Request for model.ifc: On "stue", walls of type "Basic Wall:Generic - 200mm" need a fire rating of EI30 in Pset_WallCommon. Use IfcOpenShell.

First a look at what the model holds.

```python
import ifcopenshell
import ifcopenshell.util.element

model = ifcopenshell.open("model.ifc")
print(model.schema)
storey = next(s for s in model.by_type("IfcBuildingStorey") if s.Name == "stue")
walls = [e for e in ifcopenshell.util.element.get_decomposition(storey) if e.is_a("IfcWall")]
seen = {}
for e in walls:
    element_type = ifcopenshell.util.element.get_type(e)
    key = (element_type.Name if element_type != e and element_type else None, ifcopenshell.util.element.get_pset(e, "Pset_WallCommon", "FireRating"))
    seen[key] = seen.get(key, 0) + 1
for (name, value), count in sorted(seen.items(), key=str):
    print(count, "x", name, "|", value)
```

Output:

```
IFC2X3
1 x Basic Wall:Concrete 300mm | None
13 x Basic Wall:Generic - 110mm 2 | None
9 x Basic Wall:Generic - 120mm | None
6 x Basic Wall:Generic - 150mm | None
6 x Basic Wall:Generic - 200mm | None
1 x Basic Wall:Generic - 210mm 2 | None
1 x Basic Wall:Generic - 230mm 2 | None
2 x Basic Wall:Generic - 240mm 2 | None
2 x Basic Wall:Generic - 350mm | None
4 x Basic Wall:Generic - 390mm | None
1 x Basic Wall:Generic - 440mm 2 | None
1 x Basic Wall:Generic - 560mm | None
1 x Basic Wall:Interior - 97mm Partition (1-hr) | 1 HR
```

```python
import ifcopenshell
import ifcopenshell.api.pset
import ifcopenshell.util.element

model = ifcopenshell.open("model.ifc")

storey = next(s for s in model.by_type("IfcBuildingStorey") if s.Name == "stue")
walls = [e for e in ifcopenshell.util.element.get_decomposition(storey) if e.is_a("IfcWall")]

count = 0
for e in walls:
    element_type = ifcopenshell.util.element.get_type(e)
    if element_type in (None, e) or element_type.Name != "Basic Wall:Generic - 200mm":
        continue
    # add_pset returns the element's existing set when there is one.
    pset = ifcopenshell.api.pset.add_pset(model, product=e, name="Pset_WallCommon")
    ifcopenshell.api.pset.edit_pset(model, pset=pset, properties={"FireRating": "EI30"})
    count += 1

print(count, "walls updated")

model.write("model_edited.ifc")
```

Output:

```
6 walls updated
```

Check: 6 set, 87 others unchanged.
